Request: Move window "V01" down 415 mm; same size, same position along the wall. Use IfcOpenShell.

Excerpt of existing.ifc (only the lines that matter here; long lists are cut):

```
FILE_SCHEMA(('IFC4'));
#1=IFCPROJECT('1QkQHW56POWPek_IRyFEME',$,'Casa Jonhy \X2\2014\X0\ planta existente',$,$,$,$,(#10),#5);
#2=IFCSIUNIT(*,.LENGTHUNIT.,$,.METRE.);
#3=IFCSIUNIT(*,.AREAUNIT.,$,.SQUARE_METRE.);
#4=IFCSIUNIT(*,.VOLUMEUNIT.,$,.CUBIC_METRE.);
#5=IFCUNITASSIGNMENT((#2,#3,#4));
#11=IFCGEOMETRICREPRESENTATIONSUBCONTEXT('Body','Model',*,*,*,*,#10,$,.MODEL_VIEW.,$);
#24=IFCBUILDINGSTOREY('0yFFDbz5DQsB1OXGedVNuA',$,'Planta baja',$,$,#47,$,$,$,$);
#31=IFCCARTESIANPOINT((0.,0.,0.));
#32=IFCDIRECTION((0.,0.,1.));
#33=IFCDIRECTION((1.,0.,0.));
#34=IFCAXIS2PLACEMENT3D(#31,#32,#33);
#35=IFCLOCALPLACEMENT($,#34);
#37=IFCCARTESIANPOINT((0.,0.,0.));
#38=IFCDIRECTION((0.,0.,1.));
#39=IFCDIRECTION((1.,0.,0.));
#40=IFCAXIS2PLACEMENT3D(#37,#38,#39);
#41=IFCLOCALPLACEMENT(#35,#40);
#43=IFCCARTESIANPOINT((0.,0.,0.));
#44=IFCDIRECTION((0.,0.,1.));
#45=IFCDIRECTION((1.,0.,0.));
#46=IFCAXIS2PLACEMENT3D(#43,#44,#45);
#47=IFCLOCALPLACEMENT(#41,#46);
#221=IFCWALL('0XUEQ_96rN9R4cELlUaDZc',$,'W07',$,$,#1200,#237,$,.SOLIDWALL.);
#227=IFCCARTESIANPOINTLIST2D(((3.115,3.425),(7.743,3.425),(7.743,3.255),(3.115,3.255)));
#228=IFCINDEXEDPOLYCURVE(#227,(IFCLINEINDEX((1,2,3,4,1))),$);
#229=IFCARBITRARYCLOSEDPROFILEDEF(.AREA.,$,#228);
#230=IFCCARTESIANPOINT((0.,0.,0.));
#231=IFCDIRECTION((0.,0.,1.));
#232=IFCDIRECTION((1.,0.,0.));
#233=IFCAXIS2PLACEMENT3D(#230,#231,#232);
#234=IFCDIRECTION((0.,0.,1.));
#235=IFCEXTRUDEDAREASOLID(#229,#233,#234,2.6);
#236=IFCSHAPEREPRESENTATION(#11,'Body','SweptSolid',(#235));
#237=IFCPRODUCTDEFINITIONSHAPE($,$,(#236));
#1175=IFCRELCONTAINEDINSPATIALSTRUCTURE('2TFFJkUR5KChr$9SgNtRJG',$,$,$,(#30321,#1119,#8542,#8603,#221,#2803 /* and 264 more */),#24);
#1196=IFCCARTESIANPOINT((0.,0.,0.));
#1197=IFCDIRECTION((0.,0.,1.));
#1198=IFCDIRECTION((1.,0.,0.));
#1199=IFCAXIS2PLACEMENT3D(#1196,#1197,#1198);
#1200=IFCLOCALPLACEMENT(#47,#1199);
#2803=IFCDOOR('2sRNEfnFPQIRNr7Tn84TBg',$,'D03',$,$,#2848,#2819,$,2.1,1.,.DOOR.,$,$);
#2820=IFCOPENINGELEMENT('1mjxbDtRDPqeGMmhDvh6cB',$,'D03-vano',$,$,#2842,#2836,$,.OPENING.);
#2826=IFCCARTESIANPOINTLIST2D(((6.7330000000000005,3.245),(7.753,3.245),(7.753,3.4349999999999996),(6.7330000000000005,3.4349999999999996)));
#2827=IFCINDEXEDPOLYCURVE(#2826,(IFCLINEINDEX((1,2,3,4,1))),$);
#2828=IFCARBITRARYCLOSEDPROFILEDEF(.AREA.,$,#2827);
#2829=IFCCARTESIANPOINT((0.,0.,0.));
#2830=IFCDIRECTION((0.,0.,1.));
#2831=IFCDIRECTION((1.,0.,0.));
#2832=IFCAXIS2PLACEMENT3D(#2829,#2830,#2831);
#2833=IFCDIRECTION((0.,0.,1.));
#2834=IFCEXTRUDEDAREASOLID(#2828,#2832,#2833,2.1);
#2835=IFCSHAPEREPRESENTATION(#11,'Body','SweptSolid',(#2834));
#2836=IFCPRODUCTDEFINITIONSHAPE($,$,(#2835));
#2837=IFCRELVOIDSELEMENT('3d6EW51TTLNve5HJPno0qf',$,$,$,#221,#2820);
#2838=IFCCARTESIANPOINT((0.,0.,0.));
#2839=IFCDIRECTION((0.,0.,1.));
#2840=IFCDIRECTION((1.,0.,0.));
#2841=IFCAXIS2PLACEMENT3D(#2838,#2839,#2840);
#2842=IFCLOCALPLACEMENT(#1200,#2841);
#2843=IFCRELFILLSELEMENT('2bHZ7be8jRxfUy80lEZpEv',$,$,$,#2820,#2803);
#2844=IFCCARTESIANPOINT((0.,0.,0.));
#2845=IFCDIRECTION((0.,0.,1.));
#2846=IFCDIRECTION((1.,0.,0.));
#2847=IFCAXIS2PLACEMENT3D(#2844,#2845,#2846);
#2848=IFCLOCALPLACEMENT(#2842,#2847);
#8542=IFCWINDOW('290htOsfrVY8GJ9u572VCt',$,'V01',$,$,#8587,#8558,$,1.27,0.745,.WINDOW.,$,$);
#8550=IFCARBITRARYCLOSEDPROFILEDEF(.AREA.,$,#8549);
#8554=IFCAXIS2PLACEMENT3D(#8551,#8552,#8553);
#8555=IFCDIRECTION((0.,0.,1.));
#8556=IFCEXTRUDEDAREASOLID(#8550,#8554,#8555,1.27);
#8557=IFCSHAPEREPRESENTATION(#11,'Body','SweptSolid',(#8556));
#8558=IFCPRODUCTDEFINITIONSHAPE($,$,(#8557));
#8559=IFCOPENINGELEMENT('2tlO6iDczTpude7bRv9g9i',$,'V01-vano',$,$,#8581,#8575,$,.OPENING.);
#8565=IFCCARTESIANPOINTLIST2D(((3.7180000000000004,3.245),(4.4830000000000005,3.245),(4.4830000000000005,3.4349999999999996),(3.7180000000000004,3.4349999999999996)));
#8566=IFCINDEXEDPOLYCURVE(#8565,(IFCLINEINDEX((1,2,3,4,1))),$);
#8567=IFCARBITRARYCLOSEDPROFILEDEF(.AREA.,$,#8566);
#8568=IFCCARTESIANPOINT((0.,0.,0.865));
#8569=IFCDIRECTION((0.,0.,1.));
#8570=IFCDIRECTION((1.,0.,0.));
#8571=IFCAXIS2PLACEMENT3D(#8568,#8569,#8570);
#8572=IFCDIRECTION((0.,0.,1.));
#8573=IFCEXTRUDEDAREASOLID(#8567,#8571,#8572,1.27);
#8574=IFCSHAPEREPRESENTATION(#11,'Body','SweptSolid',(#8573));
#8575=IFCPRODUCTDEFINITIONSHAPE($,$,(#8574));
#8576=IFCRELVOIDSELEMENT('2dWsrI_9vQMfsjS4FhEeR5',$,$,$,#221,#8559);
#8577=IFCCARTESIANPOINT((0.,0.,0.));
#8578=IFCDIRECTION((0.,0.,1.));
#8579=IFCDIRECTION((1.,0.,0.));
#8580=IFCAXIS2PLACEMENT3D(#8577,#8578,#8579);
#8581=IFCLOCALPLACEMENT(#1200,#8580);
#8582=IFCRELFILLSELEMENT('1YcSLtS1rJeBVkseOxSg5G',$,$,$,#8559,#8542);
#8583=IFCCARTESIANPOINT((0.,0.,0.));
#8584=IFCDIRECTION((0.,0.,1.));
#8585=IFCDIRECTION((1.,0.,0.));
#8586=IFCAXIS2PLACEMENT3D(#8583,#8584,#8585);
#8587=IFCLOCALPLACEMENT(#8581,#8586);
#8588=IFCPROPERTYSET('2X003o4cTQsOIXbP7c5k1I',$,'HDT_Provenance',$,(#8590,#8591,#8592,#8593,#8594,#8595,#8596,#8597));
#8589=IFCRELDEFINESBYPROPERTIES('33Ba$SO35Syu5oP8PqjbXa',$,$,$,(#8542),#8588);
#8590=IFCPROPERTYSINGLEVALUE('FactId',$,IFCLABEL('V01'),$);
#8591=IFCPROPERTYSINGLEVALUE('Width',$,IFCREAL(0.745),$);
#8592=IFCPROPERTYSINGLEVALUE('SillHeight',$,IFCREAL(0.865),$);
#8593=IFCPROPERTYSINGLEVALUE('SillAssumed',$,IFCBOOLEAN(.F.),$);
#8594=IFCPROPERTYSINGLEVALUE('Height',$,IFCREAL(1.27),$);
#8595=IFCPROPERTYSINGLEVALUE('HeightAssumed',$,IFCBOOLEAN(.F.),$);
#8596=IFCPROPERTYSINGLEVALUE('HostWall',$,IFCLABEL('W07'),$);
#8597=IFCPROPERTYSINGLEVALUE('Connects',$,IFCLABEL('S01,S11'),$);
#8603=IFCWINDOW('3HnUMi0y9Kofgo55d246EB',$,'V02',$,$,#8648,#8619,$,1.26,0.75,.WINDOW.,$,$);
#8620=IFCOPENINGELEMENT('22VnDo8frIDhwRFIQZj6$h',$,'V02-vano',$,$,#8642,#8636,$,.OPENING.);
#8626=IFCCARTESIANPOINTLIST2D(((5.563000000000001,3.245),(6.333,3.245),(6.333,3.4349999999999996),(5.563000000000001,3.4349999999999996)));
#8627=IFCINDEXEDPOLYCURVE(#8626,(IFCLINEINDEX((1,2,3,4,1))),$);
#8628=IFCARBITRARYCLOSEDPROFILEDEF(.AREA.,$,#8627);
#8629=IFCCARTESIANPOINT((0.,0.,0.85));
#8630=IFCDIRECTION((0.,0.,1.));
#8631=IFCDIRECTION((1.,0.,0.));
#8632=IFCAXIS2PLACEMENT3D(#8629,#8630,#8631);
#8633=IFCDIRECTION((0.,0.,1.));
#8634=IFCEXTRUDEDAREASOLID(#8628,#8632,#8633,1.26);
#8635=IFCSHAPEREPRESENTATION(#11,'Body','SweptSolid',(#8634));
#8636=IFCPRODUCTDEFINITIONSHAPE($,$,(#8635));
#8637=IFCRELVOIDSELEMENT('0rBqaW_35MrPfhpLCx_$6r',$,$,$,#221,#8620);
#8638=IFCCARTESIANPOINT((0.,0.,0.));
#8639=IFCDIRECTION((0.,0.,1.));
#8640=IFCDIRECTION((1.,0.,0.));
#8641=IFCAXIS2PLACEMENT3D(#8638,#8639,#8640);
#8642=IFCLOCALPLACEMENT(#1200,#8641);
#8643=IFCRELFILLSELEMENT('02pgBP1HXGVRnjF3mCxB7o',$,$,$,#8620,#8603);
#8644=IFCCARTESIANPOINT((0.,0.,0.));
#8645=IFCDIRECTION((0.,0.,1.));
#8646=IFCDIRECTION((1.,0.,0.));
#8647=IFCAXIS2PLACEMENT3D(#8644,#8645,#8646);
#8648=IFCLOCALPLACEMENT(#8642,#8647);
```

```python
import numpy as np
import ifcopenshell
import ifcopenshell.api.geometry
import ifcopenshell.api.pset
import ifcopenshell.util.element
import ifcopenshell.util.placement
import ifcopenshell.util.unit

model = ifcopenshell.open("existing.ifc")
unit_scale = ifcopenshell.util.unit.calculate_unit_scale(model)

window = model.by_id(8542)
opening = window.FillsVoids[0].RelatingOpeningElement
dz = -0.415

shift = np.array([0.0, 0.0, dz])
# The window is placed relative to its opening, so it follows when the opening moves.
matrix = ifcopenshell.util.placement.get_local_placement(opening.ObjectPlacement)
matrix[:3, 3] += shift
ifcopenshell.api.geometry.edit_object_placement(
    model, product=opening, matrix=matrix, is_si=False, should_transform_children=True
)

# Keep the stored heights in step.
pset = model.by_id(ifcopenshell.util.element.get_pset(window, "HDT_Provenance", should_inherit=False)["id"])
ifcopenshell.api.pset.edit_pset(model, pset=pset, properties={
    "SillHeight": model.create_entity("IfcReal", ifcopenshell.util.element.get_pset(window, "HDT_Provenance", "SillHeight") + dz),
})

print(f"moved by {dz * unit_scale:+.3f} m")

model.write("existing_edited.ifc")
```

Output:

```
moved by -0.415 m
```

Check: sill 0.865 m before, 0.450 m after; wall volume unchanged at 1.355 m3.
